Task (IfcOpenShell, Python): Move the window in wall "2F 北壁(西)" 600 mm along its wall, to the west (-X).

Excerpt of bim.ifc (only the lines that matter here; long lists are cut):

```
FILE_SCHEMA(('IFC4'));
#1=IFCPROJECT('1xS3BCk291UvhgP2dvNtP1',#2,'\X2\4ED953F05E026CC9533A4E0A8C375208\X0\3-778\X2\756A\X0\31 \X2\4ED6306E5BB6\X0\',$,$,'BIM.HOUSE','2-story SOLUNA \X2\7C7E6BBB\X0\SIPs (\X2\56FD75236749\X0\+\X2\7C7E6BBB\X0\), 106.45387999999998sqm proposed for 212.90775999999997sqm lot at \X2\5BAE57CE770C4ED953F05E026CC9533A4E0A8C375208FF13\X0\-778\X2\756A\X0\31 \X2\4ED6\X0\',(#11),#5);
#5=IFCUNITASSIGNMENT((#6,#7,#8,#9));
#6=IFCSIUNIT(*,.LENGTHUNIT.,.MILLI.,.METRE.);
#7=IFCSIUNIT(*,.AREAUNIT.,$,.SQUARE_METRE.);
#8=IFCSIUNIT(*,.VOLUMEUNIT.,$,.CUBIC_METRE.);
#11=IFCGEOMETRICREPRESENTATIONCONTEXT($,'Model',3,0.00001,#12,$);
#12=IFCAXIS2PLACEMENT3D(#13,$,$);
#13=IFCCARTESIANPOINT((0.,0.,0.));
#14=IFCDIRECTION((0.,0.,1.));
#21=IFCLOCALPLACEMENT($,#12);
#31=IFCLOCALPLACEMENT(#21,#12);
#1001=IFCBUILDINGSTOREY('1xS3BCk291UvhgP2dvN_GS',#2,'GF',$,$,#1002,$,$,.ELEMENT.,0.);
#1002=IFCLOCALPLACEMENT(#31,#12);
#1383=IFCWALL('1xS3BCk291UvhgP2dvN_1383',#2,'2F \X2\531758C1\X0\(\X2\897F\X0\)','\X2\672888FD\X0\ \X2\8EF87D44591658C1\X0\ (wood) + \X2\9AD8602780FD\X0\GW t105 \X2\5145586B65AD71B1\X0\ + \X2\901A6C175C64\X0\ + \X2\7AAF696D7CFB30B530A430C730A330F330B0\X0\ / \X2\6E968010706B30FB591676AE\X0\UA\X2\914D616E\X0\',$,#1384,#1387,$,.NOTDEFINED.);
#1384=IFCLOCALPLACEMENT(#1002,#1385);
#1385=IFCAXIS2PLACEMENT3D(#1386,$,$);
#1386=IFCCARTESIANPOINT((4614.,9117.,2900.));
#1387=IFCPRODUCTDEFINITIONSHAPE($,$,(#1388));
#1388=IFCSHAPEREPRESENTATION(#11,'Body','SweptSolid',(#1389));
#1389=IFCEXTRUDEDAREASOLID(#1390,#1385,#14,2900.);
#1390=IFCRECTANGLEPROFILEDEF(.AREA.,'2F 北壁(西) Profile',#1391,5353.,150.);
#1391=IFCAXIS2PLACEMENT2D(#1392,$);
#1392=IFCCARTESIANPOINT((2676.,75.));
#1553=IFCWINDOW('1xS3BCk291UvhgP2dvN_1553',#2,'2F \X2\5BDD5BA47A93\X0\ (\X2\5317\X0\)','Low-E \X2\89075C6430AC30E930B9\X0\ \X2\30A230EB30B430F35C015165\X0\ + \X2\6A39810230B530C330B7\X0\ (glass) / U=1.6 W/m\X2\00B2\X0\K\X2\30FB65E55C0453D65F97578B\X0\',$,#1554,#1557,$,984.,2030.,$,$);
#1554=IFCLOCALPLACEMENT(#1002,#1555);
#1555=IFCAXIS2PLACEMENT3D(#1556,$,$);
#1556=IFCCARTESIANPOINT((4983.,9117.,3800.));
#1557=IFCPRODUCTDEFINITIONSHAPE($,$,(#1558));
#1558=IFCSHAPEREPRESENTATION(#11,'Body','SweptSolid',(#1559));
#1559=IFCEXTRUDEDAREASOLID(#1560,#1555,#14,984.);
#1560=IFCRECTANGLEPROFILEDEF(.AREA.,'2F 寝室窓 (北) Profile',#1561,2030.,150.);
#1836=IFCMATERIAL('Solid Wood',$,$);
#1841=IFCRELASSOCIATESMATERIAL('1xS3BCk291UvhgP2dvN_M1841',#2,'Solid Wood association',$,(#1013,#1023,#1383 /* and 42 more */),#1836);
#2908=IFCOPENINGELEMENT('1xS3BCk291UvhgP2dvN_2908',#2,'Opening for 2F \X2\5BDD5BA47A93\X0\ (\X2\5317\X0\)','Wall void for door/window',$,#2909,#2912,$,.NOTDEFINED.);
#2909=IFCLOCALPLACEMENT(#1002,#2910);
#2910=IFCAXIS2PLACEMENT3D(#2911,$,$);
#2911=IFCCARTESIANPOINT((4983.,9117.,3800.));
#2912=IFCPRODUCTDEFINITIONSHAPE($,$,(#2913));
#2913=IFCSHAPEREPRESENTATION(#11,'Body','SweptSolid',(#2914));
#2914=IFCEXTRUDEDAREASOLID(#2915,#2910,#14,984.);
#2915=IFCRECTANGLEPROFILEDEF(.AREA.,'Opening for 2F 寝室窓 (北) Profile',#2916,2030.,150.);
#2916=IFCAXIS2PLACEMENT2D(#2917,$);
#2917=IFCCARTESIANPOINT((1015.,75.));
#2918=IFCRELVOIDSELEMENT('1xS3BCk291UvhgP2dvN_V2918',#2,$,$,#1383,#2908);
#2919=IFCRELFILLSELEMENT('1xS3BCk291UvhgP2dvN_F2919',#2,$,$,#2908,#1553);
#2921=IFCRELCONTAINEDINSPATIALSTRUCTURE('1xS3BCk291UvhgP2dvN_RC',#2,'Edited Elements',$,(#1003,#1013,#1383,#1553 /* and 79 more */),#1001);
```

```python
import ifcopenshell
import ifcopenshell.api.geometry
import ifcopenshell.util.placement
import ifcopenshell.util.unit

model = ifcopenshell.open("bim.ifc")
unit_scale = ifcopenshell.util.unit.calculate_unit_scale(model)

window = model.by_guid("1xS3BCk291UvhgP2dvN_1553")
opening = window.FillsVoids[0].RelatingOpeningElement
wall = opening.VoidsElements[0].RelatingBuildingElement

wall_matrix = ifcopenshell.util.placement.get_local_placement(wall.ObjectPlacement)
shift = wall_matrix[:3, 0] * -0.6 / unit_scale
before = ifcopenshell.util.placement.get_local_placement(window.ObjectPlacement)[:3, 3].copy()

# The window is not placed relative to its opening, so move both.
for product in (opening, window):
    matrix = ifcopenshell.util.placement.get_local_placement(product.ObjectPlacement)
    matrix[:3, 3] += shift
    ifcopenshell.api.geometry.edit_object_placement(model, product=product, matrix=matrix, is_si=False)

after = ifcopenshell.util.placement.get_local_placement(window.ObjectPlacement)[:3, 3]
print("window moved by", (after - before).round(3) + 0.0)

model.write("bim_v2.ifc")
```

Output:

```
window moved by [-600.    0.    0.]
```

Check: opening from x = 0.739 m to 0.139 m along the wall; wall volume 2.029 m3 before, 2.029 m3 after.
